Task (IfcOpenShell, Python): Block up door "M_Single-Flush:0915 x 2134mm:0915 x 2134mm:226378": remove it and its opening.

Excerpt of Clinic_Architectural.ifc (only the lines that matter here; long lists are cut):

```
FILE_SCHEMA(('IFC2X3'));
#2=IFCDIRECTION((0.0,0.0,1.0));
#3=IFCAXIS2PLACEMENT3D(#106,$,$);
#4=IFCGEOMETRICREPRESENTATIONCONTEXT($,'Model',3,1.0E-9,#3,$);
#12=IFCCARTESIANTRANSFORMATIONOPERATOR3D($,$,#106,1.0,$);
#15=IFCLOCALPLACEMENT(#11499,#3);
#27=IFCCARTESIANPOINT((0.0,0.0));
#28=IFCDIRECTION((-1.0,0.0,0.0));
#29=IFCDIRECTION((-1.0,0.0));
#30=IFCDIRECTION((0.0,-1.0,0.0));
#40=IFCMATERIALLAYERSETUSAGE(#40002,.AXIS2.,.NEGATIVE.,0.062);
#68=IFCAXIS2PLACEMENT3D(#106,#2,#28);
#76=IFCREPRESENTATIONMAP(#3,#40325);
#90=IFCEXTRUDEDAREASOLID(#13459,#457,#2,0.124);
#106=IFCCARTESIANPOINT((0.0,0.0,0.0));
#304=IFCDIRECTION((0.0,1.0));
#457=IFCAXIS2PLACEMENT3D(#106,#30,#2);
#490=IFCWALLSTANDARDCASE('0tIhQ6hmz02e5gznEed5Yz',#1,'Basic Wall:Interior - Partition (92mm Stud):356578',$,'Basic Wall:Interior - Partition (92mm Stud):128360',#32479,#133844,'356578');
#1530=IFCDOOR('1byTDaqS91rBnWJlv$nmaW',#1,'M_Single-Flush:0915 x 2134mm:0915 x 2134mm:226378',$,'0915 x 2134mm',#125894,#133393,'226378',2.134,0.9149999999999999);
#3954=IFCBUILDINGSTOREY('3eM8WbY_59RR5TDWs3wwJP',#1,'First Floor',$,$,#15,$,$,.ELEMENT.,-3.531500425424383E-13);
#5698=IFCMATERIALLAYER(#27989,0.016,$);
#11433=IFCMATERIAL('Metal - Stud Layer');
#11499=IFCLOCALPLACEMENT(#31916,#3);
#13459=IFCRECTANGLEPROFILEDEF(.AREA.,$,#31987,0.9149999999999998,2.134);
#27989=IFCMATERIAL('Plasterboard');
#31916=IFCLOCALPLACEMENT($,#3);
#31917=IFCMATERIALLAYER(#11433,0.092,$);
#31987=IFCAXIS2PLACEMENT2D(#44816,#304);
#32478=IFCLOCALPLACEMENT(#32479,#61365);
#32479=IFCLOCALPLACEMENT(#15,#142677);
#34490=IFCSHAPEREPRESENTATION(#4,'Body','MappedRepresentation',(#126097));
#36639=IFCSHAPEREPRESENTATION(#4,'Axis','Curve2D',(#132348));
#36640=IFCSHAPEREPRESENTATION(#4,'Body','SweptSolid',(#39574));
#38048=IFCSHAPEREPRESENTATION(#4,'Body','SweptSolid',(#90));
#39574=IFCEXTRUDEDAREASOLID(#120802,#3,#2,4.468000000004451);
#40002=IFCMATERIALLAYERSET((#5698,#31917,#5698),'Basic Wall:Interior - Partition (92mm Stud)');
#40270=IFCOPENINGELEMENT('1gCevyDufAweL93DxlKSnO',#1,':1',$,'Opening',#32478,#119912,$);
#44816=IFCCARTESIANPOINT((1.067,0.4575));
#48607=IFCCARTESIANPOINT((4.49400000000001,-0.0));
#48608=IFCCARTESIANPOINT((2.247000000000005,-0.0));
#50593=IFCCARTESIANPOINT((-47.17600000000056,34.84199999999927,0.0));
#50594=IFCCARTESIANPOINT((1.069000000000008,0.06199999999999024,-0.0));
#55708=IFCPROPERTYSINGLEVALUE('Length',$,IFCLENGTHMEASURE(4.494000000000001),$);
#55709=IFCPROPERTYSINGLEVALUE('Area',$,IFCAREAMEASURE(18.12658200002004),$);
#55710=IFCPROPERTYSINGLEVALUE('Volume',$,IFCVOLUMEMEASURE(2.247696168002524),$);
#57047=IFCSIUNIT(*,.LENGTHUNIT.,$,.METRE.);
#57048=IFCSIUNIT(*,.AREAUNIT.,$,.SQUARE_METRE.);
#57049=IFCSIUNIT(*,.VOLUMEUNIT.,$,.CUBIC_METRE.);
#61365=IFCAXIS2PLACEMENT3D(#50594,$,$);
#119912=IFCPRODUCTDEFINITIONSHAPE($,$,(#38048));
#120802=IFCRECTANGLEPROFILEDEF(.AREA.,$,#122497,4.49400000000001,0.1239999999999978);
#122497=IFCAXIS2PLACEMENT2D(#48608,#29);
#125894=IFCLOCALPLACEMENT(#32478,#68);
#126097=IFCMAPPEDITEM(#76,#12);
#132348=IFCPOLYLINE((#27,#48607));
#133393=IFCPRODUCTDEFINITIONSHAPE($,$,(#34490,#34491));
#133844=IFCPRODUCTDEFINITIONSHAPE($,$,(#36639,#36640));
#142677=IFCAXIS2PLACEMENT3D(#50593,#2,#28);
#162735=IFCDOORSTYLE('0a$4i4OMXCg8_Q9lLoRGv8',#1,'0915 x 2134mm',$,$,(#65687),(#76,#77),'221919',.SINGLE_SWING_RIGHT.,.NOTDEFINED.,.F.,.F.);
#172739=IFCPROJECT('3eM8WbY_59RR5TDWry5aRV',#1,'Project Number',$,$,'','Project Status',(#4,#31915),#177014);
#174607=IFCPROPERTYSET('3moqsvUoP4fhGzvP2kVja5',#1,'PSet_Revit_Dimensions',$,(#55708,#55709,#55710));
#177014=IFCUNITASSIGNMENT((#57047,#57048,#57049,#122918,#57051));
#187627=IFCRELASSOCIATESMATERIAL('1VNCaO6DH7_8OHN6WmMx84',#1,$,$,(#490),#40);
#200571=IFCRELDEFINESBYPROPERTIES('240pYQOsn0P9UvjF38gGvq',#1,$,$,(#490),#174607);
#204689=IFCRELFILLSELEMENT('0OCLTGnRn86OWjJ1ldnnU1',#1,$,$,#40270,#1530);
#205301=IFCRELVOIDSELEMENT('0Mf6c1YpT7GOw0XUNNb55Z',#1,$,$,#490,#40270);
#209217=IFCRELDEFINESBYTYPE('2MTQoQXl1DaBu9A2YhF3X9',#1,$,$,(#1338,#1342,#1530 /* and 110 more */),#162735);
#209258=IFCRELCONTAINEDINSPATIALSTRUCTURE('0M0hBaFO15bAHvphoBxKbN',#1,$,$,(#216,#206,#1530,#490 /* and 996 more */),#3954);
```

```python
import ifcopenshell
import ifcopenshell.api.feature
import ifcopenshell.api.pset
import ifcopenshell.api.root
import ifcopenshell.geom
import ifcopenshell.util.element
import ifcopenshell.util.shape
import ifcopenshell.util.unit

model = ifcopenshell.open("Clinic_Architectural.ifc")
area_scale = ifcopenshell.util.unit.calculate_unit_scale(model, "AREAUNIT")
volume_scale = ifcopenshell.util.unit.calculate_unit_scale(model, "VOLUMEUNIT")
settings = ifcopenshell.geom.settings()


def volume(element):
    """Net volume in cubic metres, openings subtracted."""
    shape = ifcopenshell.geom.create_shape(settings, element)
    return ifcopenshell.util.shape.get_volume(shape.geometry)


door = model.by_id(1530)
opening = door.FillsVoids[0].RelatingOpeningElement
wall = opening.VoidsElements[0].RelatingBuildingElement
before = volume(wall)

ifcopenshell.api.root.remove_product(model, product=door)
ifcopenshell.api.feature.remove_feature(model, feature=opening)

after = volume(wall)
thickness = 0.124  # wall thickness in metres

# Update the wall's stored quantities.
pset = model.by_id(ifcopenshell.util.element.get_pset(wall, "PSet_Revit_Dimensions", should_inherit=False)["id"])
ifcopenshell.api.pset.edit_pset(model, pset=pset, properties={
    "Area": model.create_entity("IfcAreaMeasure", after / thickness / area_scale),
    "Volume": model.create_entity("IfcVolumeMeasure", after / volume_scale),
})

print(f"wall volume {before:.3f} -> {after:.3f} m3")

model.write("Clinic_Architectural_edited.ifc")
```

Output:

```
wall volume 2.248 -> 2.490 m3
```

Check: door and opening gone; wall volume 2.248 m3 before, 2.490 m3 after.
